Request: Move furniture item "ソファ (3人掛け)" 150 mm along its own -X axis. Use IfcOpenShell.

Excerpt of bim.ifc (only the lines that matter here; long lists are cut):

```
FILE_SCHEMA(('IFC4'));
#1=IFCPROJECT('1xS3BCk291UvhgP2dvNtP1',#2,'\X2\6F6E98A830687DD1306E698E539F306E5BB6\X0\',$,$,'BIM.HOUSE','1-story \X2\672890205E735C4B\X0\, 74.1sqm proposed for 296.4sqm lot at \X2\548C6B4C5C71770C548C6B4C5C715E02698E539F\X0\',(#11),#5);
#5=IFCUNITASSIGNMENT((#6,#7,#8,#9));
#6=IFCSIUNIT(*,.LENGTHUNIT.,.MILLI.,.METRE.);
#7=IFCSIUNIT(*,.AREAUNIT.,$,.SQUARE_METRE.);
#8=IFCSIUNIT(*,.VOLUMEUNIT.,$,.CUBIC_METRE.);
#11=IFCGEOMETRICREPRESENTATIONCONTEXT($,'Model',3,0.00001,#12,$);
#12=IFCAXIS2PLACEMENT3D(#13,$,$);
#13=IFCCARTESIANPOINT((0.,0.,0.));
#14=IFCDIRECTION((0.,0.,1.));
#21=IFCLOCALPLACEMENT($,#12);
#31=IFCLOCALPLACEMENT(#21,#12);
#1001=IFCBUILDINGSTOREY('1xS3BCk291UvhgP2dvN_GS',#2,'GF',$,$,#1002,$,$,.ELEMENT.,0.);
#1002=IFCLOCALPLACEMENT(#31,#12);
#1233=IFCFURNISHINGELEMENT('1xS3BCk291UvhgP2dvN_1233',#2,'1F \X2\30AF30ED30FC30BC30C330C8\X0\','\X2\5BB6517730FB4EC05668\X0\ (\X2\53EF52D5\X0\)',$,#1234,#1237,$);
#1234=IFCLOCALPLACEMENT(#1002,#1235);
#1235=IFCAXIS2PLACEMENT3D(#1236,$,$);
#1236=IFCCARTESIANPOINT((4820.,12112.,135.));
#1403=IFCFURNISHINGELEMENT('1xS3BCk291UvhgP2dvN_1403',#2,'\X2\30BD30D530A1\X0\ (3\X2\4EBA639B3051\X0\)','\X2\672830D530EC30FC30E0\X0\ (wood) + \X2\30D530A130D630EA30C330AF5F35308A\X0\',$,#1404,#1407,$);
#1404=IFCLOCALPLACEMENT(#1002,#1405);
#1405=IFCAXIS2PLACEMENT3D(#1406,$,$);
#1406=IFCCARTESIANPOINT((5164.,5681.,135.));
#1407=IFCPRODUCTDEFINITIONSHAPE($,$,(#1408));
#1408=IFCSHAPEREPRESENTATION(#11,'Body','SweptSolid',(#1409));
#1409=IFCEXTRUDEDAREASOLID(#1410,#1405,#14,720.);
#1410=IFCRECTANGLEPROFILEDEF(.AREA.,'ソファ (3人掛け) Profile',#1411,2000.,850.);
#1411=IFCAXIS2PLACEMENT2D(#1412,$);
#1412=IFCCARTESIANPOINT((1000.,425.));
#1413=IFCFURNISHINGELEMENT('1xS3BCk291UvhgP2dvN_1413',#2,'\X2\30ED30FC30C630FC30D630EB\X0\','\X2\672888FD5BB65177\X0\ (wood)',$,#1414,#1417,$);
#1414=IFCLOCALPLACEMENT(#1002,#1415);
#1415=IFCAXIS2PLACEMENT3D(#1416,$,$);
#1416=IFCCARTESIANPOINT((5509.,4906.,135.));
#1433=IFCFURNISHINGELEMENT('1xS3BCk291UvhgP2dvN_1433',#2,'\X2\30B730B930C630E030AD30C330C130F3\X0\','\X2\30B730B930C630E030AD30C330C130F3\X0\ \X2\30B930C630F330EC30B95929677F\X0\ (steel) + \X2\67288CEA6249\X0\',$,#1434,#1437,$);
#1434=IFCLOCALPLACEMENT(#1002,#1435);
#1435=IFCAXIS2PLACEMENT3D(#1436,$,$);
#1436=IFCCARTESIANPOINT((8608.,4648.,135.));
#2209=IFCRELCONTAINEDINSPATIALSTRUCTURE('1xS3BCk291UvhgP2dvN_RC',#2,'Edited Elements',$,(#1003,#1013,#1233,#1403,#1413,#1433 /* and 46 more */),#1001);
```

```python
import ifcopenshell
import ifcopenshell.api.geometry
import ifcopenshell.util.placement
import ifcopenshell.util.unit

model = ifcopenshell.open("bim.ifc")
unit_scale = ifcopenshell.util.unit.calculate_unit_scale(model)

item = model.by_id(1403)
matrix = ifcopenshell.util.placement.get_local_placement(item.ObjectPlacement)
matrix[:3, 3] -= matrix[:3, 0] * 0.15 / unit_scale
ifcopenshell.api.geometry.edit_object_placement(model, product=item, matrix=matrix, is_si=False)

print(ifcopenshell.util.placement.get_local_placement(item.ObjectPlacement).round(3) + 0.0)

model.write("bim-out.ifc")
```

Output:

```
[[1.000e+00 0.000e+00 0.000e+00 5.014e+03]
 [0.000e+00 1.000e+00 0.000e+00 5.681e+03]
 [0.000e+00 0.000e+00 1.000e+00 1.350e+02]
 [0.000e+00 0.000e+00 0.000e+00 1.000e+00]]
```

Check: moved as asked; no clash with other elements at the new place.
